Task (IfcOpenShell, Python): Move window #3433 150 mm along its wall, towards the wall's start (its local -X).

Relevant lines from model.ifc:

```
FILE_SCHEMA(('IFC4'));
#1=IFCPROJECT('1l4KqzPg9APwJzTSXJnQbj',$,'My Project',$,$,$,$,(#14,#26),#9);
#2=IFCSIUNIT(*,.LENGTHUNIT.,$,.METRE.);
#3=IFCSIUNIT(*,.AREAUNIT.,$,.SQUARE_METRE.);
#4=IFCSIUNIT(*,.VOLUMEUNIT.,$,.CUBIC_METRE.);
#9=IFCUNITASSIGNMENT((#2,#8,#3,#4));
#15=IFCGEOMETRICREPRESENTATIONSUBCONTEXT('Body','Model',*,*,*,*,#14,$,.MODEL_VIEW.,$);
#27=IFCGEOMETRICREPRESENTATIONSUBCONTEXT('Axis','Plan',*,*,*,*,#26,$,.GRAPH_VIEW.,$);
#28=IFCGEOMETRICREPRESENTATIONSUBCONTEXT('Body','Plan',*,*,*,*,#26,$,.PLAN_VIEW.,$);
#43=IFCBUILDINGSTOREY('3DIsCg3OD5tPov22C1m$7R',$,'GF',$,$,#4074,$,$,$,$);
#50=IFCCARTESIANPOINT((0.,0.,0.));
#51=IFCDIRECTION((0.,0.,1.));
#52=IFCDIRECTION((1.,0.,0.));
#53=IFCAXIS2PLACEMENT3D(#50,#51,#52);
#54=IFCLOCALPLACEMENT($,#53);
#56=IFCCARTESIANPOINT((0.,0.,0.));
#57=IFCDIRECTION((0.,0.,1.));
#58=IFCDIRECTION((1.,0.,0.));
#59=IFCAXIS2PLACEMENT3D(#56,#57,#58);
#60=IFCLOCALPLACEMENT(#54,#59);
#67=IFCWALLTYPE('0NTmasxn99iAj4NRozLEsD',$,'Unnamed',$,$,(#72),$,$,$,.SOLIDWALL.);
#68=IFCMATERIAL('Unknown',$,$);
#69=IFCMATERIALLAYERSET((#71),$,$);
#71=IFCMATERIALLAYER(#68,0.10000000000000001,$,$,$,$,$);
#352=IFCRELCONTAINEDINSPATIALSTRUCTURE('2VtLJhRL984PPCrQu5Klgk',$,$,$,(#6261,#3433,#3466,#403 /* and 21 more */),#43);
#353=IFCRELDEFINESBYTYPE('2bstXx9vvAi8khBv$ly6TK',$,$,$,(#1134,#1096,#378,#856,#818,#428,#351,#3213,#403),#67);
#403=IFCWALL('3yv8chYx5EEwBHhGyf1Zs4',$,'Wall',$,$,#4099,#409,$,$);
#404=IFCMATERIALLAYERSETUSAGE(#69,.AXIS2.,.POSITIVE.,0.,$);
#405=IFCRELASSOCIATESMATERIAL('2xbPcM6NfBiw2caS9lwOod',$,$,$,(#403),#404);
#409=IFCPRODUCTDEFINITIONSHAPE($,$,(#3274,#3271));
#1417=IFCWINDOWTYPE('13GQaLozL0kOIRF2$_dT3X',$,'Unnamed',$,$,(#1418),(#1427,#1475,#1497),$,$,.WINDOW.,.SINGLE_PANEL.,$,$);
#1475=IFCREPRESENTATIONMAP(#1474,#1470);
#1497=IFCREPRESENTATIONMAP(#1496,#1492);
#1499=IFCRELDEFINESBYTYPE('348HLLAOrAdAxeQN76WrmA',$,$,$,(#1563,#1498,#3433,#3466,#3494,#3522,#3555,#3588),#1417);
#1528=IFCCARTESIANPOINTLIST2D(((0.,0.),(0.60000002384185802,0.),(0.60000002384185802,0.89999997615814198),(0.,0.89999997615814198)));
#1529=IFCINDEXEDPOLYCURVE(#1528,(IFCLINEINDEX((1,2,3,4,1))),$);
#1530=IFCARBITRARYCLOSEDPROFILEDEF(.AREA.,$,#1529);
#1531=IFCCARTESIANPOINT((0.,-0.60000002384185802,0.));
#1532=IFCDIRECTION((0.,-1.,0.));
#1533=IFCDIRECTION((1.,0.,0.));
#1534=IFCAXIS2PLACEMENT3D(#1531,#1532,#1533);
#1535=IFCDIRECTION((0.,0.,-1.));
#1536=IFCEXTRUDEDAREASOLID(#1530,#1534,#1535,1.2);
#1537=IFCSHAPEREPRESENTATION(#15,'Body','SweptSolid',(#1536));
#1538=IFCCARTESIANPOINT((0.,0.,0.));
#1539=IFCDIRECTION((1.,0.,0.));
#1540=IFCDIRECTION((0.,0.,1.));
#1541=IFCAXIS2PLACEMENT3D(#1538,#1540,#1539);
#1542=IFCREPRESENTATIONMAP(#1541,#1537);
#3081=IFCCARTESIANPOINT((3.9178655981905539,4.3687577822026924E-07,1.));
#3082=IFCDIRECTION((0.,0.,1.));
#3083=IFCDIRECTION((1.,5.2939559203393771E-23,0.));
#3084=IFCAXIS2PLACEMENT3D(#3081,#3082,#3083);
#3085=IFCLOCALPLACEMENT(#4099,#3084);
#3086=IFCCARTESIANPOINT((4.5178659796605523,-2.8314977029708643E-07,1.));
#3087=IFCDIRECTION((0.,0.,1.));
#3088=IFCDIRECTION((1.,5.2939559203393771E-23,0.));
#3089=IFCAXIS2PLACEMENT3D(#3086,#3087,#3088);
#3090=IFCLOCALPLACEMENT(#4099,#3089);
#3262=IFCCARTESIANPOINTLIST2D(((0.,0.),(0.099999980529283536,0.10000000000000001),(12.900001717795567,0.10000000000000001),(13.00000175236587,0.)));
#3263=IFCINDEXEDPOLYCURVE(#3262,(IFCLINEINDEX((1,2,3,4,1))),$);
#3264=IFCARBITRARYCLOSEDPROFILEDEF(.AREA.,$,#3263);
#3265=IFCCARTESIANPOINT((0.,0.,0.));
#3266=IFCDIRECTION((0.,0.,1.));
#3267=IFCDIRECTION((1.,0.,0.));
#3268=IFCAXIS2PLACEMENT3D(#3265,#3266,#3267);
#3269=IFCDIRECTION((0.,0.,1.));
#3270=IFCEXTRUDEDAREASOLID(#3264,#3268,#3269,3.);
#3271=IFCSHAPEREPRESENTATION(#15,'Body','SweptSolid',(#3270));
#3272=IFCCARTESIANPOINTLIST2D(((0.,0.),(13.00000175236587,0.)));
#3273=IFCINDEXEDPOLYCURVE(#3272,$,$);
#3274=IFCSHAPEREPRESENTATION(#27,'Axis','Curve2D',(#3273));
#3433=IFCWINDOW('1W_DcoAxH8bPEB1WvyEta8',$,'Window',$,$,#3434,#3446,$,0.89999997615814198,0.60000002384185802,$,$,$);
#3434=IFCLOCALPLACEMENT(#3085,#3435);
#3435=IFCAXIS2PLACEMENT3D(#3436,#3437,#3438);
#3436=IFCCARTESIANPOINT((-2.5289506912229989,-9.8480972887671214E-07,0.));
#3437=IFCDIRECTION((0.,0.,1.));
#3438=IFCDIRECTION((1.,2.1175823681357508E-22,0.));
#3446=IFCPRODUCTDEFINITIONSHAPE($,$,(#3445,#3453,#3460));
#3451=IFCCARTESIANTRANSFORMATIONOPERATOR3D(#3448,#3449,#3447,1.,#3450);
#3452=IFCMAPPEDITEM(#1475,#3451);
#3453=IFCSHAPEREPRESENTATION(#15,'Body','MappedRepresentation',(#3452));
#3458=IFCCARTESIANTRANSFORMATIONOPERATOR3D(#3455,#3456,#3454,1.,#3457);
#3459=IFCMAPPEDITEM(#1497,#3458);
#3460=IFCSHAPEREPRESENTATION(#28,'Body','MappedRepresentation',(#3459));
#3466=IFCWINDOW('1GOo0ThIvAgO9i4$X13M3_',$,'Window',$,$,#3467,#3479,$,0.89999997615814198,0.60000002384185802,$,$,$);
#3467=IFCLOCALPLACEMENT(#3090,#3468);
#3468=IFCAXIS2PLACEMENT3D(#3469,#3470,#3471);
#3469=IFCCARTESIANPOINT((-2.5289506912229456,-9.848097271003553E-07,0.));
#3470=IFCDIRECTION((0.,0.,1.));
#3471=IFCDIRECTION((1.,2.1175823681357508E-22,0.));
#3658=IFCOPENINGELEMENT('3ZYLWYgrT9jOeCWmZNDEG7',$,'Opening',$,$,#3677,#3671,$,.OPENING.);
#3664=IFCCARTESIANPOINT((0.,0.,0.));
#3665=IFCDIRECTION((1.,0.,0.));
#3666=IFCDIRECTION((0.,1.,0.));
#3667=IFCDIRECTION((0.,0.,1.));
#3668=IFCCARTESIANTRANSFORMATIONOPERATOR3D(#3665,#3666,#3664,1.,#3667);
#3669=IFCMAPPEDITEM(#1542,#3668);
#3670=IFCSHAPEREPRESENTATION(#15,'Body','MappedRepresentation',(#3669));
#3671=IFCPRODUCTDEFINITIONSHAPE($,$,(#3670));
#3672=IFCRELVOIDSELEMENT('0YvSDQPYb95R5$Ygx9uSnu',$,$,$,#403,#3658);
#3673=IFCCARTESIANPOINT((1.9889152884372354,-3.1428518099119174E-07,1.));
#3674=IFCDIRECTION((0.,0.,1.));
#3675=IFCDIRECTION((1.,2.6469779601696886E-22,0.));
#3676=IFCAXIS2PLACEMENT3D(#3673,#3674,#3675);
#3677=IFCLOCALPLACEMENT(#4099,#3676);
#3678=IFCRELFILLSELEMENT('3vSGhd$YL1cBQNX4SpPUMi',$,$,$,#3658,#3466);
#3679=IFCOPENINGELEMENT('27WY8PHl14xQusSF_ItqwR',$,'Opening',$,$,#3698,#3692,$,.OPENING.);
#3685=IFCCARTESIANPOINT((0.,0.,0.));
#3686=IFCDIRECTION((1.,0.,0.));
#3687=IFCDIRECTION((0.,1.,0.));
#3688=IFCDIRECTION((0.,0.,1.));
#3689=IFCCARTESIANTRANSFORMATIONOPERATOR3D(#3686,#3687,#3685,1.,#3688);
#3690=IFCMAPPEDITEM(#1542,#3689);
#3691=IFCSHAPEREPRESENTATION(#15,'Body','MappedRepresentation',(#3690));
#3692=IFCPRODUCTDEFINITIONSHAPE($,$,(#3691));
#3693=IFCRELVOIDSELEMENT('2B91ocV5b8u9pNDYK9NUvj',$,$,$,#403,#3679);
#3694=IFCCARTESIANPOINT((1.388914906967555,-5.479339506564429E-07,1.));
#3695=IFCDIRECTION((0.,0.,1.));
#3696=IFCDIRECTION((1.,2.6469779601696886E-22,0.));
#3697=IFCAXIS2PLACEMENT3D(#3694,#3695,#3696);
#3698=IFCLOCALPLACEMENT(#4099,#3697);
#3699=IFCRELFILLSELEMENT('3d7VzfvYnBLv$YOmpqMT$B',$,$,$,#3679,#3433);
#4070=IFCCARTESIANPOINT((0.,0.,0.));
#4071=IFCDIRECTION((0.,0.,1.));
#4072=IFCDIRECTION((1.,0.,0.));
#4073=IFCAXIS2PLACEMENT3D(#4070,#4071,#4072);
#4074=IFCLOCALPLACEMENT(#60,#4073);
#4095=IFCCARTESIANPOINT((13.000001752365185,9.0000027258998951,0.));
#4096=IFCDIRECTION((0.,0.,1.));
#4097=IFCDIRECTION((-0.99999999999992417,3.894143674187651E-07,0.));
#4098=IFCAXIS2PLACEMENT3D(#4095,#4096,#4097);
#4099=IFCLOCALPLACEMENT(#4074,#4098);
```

```python
import ifcopenshell
import ifcopenshell.api.geometry
import ifcopenshell.util.placement
import ifcopenshell.util.unit

model = ifcopenshell.open("model.ifc")
unit_scale = ifcopenshell.util.unit.calculate_unit_scale(model)

window = model.by_guid("1W_DcoAxH8bPEB1WvyEta8")
opening = window.FillsVoids[0].RelatingOpeningElement
wall = opening.VoidsElements[0].RelatingBuildingElement

wall_matrix = ifcopenshell.util.placement.get_local_placement(wall.ObjectPlacement)
shift = wall_matrix[:3, 0] * -0.15 / unit_scale
before = ifcopenshell.util.placement.get_local_placement(window.ObjectPlacement)[:3, 3].copy()

# The window is not placed relative to its opening, so move both.
for product in (opening, window):
    matrix = ifcopenshell.util.placement.get_local_placement(product.ObjectPlacement)
    matrix[:3, 3] += shift
    ifcopenshell.api.geometry.edit_object_placement(model, product=product, matrix=matrix, is_si=False)

after = ifcopenshell.util.placement.get_local_placement(window.ObjectPlacement)[:3, 3]
print("window moved by", (after - before).round(3) + 0.0)

model.write("model-out.ifc")
```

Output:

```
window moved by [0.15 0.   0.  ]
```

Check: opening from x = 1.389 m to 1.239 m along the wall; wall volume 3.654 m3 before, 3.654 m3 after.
